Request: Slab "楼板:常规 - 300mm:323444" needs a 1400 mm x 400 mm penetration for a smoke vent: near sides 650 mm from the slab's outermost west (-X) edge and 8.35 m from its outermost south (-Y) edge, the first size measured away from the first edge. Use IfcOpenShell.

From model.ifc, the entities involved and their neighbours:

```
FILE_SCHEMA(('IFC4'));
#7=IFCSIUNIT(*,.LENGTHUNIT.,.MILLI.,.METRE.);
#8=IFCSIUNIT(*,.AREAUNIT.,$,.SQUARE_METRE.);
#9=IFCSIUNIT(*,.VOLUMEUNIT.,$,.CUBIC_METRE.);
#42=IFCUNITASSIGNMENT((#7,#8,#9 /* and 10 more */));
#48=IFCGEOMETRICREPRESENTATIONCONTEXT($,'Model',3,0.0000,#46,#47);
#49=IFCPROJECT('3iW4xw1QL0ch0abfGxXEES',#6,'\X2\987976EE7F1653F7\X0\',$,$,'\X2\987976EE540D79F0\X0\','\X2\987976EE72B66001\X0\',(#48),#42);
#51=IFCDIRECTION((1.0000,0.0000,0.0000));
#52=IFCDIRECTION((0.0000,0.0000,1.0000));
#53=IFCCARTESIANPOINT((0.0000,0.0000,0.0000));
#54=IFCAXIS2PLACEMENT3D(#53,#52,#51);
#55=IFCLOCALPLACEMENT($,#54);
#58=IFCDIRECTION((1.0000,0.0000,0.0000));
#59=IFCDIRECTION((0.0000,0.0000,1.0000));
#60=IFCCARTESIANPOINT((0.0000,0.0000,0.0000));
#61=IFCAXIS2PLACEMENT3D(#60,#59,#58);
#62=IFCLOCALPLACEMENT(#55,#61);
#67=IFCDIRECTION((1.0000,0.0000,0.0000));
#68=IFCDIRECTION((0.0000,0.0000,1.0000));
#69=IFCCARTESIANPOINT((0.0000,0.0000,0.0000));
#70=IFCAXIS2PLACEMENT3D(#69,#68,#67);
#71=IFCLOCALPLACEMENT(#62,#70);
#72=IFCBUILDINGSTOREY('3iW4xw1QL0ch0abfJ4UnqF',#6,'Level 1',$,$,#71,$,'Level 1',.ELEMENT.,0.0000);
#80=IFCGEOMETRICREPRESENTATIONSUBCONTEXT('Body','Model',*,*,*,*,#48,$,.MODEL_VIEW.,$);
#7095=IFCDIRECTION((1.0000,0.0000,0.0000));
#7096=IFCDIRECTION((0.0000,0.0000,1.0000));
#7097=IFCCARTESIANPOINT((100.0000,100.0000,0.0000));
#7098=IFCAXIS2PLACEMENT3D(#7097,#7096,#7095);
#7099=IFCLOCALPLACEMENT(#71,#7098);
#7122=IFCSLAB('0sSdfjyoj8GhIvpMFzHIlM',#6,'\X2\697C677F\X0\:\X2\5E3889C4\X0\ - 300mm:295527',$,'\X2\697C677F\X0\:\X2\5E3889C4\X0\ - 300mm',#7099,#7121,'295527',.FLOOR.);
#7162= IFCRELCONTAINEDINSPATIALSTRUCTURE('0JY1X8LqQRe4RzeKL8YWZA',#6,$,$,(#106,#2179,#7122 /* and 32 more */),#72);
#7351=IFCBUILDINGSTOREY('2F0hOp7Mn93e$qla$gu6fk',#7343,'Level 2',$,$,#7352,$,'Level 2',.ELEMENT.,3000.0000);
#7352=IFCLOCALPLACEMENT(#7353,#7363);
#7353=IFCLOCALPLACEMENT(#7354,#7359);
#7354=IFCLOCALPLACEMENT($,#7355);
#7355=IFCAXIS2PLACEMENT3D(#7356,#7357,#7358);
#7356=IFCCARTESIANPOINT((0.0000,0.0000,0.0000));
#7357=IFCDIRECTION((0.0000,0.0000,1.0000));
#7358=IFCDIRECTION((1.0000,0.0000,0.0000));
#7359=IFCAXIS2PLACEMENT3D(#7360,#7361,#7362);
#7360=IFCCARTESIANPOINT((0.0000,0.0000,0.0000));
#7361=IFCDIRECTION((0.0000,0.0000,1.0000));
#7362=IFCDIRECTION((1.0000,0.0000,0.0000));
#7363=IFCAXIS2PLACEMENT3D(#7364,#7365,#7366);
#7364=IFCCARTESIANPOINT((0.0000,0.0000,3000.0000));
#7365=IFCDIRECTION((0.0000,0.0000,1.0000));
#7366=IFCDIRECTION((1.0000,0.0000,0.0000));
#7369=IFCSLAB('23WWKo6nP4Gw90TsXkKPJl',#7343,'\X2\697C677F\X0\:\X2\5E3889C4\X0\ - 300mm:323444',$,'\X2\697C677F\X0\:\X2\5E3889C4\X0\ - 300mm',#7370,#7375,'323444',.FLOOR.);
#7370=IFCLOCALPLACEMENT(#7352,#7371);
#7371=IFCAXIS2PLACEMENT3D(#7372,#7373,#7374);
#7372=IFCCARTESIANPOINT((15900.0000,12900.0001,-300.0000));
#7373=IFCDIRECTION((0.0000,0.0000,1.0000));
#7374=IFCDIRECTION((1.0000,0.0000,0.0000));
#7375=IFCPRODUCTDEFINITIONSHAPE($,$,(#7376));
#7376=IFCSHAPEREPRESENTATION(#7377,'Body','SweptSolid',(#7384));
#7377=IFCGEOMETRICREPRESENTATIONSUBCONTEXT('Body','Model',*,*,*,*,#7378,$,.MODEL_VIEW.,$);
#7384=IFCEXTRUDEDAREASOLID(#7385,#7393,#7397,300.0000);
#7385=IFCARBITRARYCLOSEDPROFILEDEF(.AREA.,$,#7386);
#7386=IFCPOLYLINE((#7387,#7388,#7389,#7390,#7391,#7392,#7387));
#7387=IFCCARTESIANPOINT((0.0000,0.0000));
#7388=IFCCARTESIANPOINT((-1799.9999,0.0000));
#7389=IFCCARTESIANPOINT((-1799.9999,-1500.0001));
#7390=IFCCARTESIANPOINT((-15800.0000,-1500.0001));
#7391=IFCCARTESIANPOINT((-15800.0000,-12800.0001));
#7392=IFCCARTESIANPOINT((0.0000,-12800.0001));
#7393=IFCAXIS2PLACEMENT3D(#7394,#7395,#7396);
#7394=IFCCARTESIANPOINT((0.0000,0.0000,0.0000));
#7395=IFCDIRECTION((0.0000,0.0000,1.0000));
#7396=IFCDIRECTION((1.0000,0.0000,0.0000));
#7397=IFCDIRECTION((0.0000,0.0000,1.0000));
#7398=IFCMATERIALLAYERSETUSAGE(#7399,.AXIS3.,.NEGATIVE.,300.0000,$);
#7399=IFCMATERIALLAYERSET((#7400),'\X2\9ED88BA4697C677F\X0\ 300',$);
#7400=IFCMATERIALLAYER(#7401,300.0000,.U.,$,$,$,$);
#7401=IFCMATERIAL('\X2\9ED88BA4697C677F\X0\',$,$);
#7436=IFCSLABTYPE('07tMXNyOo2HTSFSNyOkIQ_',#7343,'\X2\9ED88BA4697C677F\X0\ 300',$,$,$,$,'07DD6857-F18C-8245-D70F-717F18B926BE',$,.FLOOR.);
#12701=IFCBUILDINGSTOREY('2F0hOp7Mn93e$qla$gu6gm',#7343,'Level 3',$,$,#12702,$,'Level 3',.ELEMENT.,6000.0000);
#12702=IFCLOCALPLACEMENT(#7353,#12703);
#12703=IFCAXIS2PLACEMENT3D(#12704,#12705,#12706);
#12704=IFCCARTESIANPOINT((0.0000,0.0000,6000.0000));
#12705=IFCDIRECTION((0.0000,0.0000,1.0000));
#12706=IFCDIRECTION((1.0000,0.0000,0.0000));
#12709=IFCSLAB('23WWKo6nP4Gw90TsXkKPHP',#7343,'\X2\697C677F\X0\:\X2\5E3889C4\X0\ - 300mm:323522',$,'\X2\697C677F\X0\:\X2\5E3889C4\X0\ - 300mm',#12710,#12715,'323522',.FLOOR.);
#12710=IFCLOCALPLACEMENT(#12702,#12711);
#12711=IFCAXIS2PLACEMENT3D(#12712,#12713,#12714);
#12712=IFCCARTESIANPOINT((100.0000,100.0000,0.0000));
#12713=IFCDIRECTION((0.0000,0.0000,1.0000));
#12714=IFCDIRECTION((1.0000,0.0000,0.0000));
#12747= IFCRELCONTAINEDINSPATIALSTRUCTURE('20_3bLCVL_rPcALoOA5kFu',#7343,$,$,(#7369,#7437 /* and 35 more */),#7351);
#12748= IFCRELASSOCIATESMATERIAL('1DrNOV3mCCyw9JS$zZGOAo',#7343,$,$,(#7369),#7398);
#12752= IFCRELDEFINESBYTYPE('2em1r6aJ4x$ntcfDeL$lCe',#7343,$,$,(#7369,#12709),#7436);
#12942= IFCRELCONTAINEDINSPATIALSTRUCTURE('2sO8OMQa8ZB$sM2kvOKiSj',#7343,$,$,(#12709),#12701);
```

```python
import numpy as np
import ifcopenshell
import ifcopenshell.api.feature
import ifcopenshell.api.geometry
import ifcopenshell.api.root
import ifcopenshell.geom
import ifcopenshell.util.placement
import ifcopenshell.util.representation
import ifcopenshell.util.shape
import ifcopenshell.util.unit

model = ifcopenshell.open("model.ifc")
unit_scale = ifcopenshell.util.unit.calculate_unit_scale(model)
settings = ifcopenshell.geom.settings()


def volume(element):
    """Net volume in cubic metres, openings subtracted."""
    shape = ifcopenshell.geom.create_shape(settings, element)
    return ifcopenshell.util.shape.get_volume(shape.geometry)


slab = model.by_guid("23WWKo6nP4Gw90TsXkKPJl")
before = volume(slab)

# Extent in the slab's own axes, in metres. The edges named are its -X and -Y sides.
slab_shape = ifcopenshell.geom.create_shape(settings, slab)
vertices = ifcopenshell.util.shape.get_vertices(slab_shape.geometry)
x_min, y_min, bottom = vertices.min(axis=0)
top = vertices[:, 2].max()

opening = ifcopenshell.api.root.create_entity(model, ifc_class="IfcOpeningElement", name="Smoke vent opening", predefined_type="OPENING")
context = ifcopenshell.util.representation.get_context(model, "Model", "Body", "MODEL_VIEW")
width, depth = 1.4, 0.4
outline = [(0.0, 0.0), (width, 0.0), (width, depth), (0.0, depth), (0.0, 0.0)]
# Overshoot both faces by 50 mm so the cut is clean.
shape = ifcopenshell.api.geometry.add_slab_representation(
    model, context=context, depth=top - bottom + 0.1, polyline=outline
)
ifcopenshell.api.geometry.assign_representation(model, product=opening, representation=shape)

matrix = ifcopenshell.util.placement.get_local_placement(slab.ObjectPlacement)
matrix[:, 3] = matrix @ np.append(np.array([x_min + 0.65, y_min + 8.35, bottom - 0.05]) / unit_scale, 1.0)
ifcopenshell.api.geometry.edit_object_placement(model, product=opening, matrix=matrix, is_si=False)
ifcopenshell.api.feature.add_feature(model, feature=opening, element=slab)

after = volume(slab)

print(f"slab volume {before:.3f} -> {after:.3f} m3")

model.write("model_rev.ifc")
```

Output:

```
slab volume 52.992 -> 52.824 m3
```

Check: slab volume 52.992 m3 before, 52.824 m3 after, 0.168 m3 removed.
